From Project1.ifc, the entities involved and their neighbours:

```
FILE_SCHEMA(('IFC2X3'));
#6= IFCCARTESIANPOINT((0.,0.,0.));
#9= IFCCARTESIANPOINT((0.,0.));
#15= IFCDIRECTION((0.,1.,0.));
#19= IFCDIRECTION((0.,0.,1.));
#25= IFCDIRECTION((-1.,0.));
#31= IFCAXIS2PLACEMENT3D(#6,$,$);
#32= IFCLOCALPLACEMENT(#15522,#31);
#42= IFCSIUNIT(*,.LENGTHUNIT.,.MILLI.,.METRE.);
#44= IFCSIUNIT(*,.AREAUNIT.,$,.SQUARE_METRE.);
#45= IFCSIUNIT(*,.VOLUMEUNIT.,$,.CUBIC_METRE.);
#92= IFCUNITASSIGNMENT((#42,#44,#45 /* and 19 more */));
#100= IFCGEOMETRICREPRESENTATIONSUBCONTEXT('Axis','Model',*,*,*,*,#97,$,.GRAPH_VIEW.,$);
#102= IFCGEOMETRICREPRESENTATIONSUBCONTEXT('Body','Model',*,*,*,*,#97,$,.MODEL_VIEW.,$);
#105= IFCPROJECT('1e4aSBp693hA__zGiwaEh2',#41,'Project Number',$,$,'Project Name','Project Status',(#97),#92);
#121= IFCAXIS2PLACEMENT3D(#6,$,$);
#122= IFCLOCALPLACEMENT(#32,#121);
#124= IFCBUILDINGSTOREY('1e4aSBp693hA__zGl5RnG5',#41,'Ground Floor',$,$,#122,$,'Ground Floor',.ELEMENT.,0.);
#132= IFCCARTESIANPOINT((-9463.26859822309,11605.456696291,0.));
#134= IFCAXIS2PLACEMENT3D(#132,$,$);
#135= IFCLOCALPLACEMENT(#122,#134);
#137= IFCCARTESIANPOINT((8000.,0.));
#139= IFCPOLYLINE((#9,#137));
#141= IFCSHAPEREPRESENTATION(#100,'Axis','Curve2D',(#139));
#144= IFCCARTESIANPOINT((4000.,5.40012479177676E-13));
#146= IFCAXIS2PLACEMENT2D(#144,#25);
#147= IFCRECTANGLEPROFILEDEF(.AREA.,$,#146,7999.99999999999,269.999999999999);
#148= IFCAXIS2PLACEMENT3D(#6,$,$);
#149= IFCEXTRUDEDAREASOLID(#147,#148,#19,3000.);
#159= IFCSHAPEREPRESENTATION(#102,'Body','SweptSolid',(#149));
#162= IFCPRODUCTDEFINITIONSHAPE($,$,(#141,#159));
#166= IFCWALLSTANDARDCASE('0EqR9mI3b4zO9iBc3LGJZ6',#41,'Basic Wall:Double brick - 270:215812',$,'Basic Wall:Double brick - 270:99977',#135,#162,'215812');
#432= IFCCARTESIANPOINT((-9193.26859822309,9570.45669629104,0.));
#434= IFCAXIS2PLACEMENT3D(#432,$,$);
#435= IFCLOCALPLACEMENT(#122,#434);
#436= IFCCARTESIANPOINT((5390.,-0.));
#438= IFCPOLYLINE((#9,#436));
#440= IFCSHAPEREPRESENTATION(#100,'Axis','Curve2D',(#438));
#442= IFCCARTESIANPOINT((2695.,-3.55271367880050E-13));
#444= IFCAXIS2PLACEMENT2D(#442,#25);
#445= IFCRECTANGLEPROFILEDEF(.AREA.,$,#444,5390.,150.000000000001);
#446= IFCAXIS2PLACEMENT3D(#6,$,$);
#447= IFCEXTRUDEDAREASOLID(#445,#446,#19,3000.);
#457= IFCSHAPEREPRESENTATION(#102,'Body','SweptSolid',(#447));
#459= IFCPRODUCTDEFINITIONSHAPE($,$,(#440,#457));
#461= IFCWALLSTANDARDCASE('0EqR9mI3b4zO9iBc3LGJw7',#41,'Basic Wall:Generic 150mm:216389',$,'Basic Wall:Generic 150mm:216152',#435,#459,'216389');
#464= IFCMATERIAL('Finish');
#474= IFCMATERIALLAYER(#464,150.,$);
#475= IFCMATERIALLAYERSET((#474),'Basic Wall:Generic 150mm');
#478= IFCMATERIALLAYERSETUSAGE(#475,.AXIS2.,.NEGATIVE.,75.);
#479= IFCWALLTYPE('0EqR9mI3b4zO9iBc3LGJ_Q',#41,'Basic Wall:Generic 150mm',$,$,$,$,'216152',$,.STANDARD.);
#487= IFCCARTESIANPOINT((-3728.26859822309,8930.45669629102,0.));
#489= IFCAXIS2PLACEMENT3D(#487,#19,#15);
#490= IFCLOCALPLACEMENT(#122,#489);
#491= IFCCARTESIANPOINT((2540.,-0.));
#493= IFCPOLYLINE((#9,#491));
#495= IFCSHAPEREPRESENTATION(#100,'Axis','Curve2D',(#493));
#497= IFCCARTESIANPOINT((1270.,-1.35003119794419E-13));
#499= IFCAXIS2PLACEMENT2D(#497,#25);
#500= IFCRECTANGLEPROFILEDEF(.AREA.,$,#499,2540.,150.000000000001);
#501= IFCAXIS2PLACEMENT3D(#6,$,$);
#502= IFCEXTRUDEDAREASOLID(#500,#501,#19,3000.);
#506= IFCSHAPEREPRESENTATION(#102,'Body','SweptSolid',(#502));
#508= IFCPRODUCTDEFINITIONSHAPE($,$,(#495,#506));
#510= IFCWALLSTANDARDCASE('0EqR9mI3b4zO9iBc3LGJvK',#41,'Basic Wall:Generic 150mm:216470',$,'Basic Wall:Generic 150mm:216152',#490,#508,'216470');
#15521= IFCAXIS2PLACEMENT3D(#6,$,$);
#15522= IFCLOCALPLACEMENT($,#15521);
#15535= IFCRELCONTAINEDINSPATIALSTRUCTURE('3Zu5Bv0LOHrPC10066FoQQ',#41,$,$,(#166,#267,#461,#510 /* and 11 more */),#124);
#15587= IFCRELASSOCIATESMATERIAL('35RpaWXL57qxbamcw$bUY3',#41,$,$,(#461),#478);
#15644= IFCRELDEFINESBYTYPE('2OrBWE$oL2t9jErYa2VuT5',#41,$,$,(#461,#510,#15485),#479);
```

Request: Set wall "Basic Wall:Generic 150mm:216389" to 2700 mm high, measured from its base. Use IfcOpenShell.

```python
import ifcopenshell
import ifcopenshell.geom
import ifcopenshell.util.representation
import ifcopenshell.util.shape
import ifcopenshell.util.unit

model = ifcopenshell.open("Project1.ifc")
unit_scale = ifcopenshell.util.unit.calculate_unit_scale(model)
settings = ifcopenshell.geom.settings()


def volume(element):
    """Net volume in cubic metres, openings subtracted."""
    shape = ifcopenshell.geom.create_shape(settings, element)
    return ifcopenshell.util.shape.get_volume(shape.geometry)


wall = model.by_id(461)
before = volume(wall)

body = ifcopenshell.util.representation.get_representation(wall, "Model", "Body")
solid = body.Items[0]
old_height = solid.Depth
solid.Depth = 2.7 / unit_scale
after = volume(wall)

print(f"height {old_height:g} -> {solid.Depth:g}, volume {before:.3f} -> {after:.3f} m3")

model.write("Project1_updated.ifc")
```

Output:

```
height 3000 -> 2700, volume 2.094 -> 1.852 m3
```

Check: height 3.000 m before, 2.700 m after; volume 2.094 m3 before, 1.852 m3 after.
